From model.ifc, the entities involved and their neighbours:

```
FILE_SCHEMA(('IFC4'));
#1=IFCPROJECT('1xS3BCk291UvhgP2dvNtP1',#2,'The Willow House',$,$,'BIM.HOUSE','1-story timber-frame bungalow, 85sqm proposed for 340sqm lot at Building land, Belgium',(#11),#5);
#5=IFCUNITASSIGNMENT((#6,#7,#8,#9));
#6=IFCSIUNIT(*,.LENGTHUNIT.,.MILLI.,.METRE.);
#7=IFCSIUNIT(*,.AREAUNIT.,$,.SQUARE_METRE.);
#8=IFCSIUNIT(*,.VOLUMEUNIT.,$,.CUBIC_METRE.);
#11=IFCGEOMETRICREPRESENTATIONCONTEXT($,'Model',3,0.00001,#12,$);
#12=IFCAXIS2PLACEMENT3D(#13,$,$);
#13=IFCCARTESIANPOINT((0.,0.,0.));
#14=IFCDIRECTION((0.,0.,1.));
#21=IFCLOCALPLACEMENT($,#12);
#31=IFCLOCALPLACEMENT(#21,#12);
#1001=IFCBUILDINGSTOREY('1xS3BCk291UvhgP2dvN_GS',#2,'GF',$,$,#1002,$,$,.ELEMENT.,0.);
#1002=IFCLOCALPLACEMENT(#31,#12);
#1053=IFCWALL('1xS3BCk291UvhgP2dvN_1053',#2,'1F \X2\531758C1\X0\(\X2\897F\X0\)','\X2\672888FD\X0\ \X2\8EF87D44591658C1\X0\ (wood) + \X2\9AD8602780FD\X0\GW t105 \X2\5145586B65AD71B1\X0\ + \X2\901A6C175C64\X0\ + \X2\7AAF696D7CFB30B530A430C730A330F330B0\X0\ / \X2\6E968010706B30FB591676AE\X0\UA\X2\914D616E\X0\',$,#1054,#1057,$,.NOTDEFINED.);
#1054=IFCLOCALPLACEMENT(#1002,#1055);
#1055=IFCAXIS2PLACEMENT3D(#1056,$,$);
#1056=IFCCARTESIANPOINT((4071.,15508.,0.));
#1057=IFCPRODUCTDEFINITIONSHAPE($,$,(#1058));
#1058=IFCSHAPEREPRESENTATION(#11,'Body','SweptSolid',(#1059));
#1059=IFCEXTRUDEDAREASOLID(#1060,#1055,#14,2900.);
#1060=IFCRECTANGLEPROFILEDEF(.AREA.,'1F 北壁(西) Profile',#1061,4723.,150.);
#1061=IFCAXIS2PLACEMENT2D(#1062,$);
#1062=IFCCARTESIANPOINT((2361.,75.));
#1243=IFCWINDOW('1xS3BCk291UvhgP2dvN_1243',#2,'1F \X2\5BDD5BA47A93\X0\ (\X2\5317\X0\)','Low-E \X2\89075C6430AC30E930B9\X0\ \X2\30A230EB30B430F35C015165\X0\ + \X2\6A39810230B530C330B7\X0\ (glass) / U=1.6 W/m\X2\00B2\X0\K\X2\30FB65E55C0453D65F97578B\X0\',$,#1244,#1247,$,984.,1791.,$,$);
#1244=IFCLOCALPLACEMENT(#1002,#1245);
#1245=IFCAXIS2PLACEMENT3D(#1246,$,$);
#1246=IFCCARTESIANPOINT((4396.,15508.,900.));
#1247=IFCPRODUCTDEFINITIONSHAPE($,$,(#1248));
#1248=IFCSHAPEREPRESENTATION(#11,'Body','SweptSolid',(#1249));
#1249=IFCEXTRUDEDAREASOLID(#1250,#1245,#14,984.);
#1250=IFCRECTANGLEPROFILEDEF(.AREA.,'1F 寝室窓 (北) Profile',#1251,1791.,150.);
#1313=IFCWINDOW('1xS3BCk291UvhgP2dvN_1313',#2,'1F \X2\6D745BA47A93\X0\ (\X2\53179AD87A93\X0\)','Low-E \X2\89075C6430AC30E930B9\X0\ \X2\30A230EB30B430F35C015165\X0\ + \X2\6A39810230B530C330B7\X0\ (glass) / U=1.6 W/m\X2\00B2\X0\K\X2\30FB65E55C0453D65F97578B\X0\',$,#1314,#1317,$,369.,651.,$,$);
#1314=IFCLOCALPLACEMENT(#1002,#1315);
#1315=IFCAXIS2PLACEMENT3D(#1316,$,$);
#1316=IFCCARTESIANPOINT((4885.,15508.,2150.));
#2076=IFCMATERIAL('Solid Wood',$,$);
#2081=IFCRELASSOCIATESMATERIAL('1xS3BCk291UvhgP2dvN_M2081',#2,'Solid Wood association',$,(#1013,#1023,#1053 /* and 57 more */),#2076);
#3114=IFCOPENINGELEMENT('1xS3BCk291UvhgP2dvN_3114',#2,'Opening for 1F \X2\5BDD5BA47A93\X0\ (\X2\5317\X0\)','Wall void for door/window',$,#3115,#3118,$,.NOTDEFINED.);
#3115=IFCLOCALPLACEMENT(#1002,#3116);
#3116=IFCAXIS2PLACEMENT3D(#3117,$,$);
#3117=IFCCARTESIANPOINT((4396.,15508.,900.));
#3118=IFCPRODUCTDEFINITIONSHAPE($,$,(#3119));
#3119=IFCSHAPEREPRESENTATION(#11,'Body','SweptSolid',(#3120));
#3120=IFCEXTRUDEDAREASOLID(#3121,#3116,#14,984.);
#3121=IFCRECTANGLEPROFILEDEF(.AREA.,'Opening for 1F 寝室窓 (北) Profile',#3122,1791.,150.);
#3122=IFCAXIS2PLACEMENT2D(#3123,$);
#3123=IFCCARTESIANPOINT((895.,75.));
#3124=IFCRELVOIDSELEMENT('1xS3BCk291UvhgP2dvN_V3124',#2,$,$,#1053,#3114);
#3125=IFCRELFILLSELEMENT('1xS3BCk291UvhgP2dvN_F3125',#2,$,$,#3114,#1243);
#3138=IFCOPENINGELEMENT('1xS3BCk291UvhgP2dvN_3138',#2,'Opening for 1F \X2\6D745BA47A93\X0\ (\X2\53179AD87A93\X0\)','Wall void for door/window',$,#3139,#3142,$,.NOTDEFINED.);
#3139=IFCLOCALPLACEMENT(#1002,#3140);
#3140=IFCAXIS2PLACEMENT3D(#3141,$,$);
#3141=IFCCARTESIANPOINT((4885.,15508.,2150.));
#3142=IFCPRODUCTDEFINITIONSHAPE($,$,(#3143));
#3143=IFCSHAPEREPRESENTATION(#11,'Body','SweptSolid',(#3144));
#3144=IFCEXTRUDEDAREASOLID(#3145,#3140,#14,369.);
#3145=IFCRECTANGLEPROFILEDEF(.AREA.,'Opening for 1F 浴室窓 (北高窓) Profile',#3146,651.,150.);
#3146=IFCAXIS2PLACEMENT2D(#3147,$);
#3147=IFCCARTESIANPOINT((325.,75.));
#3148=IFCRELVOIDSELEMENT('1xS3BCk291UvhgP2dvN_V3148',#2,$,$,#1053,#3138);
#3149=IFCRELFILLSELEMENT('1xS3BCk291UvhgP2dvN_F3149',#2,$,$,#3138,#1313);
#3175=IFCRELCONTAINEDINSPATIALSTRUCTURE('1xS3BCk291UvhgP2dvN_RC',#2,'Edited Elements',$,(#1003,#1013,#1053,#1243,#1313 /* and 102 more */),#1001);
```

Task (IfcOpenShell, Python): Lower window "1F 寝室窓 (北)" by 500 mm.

```python
import numpy as np
import ifcopenshell
import ifcopenshell.api.geometry
import ifcopenshell.util.placement
import ifcopenshell.util.unit

model = ifcopenshell.open("model.ifc")
unit_scale = ifcopenshell.util.unit.calculate_unit_scale(model)

window = model.by_guid("1xS3BCk291UvhgP2dvN_1243")
opening = window.FillsVoids[0].RelatingOpeningElement
dz = -500.0

shift = np.array([0.0, 0.0, dz])
# The window is not placed relative to its opening, so move both.
for product in (opening, window):
    matrix = ifcopenshell.util.placement.get_local_placement(product.ObjectPlacement)
    matrix[:3, 3] += shift
    ifcopenshell.api.geometry.edit_object_placement(model, product=product, matrix=matrix, is_si=False)

print(f"moved by {dz * unit_scale:+.3f} m")

model.write("model_v2.ifc")
```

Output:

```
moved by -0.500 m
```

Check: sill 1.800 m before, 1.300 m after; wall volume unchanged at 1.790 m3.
